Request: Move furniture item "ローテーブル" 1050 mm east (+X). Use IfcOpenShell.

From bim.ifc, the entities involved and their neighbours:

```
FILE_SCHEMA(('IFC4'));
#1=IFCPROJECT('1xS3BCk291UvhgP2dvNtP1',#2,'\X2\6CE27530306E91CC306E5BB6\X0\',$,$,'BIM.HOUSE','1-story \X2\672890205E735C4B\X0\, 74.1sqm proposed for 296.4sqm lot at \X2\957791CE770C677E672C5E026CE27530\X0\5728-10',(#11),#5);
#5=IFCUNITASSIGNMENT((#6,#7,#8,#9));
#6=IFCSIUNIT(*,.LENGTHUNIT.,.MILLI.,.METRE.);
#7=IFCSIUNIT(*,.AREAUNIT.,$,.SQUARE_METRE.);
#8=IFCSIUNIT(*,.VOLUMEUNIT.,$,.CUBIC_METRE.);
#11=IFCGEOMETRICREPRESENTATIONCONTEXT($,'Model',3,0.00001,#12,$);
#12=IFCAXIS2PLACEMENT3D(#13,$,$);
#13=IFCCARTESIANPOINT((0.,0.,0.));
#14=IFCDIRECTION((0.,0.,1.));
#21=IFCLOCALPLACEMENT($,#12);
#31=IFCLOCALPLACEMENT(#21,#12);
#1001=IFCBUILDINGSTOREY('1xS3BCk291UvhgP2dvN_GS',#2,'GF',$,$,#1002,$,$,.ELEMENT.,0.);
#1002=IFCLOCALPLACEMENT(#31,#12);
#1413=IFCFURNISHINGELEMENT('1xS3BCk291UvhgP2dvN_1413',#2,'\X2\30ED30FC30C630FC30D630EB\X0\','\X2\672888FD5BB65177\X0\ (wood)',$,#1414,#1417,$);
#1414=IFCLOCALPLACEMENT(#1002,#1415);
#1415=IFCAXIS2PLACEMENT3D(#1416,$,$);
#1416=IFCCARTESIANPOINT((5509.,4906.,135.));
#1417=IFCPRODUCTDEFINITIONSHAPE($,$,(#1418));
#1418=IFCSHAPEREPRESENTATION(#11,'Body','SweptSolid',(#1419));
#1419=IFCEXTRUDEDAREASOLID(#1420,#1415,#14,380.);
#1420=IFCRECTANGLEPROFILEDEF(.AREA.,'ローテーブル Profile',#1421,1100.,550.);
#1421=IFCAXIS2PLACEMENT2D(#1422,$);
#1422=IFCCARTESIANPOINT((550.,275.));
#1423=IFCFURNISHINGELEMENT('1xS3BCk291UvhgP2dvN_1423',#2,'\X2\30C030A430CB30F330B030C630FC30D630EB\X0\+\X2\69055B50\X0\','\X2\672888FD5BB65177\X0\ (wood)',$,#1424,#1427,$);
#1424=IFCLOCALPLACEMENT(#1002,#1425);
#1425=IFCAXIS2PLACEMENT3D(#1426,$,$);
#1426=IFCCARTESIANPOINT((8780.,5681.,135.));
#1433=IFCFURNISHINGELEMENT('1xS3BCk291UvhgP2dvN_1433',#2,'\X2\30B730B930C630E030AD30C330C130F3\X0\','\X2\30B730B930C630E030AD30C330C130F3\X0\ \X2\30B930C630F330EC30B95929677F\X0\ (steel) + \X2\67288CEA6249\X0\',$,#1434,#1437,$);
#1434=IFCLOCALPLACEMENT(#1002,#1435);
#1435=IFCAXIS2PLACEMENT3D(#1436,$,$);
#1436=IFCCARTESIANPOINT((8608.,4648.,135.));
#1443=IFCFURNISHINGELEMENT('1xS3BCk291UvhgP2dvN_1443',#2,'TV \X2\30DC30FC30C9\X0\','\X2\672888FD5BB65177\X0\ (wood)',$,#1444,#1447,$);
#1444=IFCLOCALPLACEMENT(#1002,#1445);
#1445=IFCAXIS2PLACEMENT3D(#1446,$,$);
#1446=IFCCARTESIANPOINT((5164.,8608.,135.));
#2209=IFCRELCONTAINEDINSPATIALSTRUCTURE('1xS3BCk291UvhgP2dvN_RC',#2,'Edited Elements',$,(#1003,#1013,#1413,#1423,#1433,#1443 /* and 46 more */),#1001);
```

```python
import ifcopenshell
import ifcopenshell.api.geometry
import ifcopenshell.util.placement
import ifcopenshell.util.unit

model = ifcopenshell.open("bim.ifc")
unit_scale = ifcopenshell.util.unit.calculate_unit_scale(model)

item = model.by_guid("1xS3BCk291UvhgP2dvN_1413")
matrix = ifcopenshell.util.placement.get_local_placement(item.ObjectPlacement)
matrix[0, 3] += 1.05 / unit_scale
ifcopenshell.api.geometry.edit_object_placement(model, product=item, matrix=matrix, is_si=False)

print(ifcopenshell.util.placement.get_local_placement(item.ObjectPlacement).round(3) + 0.0)

model.write("bim_rev.ifc")
```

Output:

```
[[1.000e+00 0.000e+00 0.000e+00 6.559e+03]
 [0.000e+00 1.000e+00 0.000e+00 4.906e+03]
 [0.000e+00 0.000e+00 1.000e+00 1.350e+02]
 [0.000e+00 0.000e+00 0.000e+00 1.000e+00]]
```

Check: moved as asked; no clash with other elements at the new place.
